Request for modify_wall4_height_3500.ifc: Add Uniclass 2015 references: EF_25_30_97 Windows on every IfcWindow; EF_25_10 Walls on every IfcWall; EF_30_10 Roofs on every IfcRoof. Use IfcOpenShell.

First a look at what the model holds.

```python
import ifcopenshell

model = ifcopenshell.open("modify_wall4_height_3500.ifc")
print(model.schema)
print("classifications:", [c.Name for c in model.by_type("IfcClassification")])
for ifc_class in ("IfcDoor", "IfcRoof", "IfcStair", "IfcWall", "IfcWindow"):
    print(ifc_class, len(model.by_type(ifc_class)))
```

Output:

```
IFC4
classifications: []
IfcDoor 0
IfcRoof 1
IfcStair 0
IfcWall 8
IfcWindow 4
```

```python
import ifcopenshell
import ifcopenshell.api.classification

model = ifcopenshell.open("modify_wall4_height_3500.ifc")

system = ifcopenshell.api.classification.add_classification(model, classification="Uniclass 2015")

codes = {
    "IfcWindow": ("EF_25_30_97", "Windows"),
    "IfcWall": ("EF_25_10", "Walls"),
    "IfcRoof": ("EF_30_10", "Roofs"),
}
for ifc_class, (code, name) in codes.items():
    products = model.by_type(ifc_class)
    ifcopenshell.api.classification.add_reference(
        model, products=products, classification=system, identification=code, name=name
    )
    print(code, len(products))

model.write("modify_wall4_height_3500_edited.ifc")
```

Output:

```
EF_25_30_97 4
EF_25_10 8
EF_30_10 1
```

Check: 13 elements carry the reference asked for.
